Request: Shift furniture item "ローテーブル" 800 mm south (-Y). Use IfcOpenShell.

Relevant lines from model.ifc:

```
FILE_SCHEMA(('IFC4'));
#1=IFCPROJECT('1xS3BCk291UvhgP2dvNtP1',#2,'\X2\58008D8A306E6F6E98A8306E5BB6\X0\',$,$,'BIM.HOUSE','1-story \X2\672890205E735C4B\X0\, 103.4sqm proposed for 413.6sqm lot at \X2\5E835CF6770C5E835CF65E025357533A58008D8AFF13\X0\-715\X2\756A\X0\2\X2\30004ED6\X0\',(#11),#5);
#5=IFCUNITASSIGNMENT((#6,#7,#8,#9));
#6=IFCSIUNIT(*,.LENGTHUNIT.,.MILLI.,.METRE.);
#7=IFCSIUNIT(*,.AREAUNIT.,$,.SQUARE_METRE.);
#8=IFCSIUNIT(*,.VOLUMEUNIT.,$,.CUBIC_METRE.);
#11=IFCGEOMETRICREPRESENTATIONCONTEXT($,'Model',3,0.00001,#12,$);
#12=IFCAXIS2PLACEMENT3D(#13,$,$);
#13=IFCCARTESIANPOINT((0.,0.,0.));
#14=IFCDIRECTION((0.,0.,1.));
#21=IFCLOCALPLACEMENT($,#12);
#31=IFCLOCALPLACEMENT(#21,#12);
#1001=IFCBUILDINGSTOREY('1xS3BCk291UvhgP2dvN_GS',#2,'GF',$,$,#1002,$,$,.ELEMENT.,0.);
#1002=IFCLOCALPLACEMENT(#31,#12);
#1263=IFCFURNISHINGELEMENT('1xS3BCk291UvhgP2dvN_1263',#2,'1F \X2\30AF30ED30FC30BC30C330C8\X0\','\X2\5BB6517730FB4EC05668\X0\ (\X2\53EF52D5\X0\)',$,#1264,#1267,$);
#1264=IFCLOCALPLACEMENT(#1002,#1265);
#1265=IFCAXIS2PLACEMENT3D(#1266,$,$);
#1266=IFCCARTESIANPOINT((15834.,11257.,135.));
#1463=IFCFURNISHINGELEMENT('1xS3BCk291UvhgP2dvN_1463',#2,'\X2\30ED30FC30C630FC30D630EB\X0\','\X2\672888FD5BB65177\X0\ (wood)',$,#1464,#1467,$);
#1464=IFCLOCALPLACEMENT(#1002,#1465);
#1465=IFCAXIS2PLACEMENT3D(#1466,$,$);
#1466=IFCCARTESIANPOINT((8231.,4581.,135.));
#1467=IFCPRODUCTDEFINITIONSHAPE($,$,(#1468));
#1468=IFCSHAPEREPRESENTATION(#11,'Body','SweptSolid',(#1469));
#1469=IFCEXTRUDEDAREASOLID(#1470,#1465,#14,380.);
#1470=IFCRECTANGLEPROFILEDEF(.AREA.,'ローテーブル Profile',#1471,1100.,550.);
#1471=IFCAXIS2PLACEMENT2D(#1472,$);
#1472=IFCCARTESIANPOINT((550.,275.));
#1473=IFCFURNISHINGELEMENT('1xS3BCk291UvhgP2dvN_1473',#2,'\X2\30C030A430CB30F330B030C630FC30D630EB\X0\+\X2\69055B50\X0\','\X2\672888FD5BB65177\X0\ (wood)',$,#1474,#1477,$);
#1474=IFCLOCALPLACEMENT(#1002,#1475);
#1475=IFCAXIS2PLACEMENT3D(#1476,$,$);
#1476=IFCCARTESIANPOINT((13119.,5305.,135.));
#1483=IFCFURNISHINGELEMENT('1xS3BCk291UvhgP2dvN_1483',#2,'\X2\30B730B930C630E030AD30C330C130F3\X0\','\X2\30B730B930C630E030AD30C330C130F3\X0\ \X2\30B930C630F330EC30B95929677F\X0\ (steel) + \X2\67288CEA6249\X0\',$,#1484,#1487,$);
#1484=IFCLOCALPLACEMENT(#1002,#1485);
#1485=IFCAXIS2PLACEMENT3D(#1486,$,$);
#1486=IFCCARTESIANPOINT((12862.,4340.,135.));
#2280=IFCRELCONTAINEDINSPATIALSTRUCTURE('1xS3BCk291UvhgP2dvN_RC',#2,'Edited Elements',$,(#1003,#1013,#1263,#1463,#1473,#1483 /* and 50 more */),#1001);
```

```python
import ifcopenshell
import ifcopenshell.api.geometry
import ifcopenshell.util.placement

model = ifcopenshell.open("model.ifc")

item = model.by_guid("1xS3BCk291UvhgP2dvN_1463")
matrix = ifcopenshell.util.placement.get_local_placement(item.ObjectPlacement)
matrix[1, 3] -= 800.0
ifcopenshell.api.geometry.edit_object_placement(model, product=item, matrix=matrix, is_si=False)

print(ifcopenshell.util.placement.get_local_placement(item.ObjectPlacement).round(3) + 0.0)

model.write("model_edited.ifc")
```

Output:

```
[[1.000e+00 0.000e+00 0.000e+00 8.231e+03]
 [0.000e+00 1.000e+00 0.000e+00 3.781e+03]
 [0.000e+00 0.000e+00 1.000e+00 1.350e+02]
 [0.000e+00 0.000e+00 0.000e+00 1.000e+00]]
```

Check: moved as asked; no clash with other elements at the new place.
